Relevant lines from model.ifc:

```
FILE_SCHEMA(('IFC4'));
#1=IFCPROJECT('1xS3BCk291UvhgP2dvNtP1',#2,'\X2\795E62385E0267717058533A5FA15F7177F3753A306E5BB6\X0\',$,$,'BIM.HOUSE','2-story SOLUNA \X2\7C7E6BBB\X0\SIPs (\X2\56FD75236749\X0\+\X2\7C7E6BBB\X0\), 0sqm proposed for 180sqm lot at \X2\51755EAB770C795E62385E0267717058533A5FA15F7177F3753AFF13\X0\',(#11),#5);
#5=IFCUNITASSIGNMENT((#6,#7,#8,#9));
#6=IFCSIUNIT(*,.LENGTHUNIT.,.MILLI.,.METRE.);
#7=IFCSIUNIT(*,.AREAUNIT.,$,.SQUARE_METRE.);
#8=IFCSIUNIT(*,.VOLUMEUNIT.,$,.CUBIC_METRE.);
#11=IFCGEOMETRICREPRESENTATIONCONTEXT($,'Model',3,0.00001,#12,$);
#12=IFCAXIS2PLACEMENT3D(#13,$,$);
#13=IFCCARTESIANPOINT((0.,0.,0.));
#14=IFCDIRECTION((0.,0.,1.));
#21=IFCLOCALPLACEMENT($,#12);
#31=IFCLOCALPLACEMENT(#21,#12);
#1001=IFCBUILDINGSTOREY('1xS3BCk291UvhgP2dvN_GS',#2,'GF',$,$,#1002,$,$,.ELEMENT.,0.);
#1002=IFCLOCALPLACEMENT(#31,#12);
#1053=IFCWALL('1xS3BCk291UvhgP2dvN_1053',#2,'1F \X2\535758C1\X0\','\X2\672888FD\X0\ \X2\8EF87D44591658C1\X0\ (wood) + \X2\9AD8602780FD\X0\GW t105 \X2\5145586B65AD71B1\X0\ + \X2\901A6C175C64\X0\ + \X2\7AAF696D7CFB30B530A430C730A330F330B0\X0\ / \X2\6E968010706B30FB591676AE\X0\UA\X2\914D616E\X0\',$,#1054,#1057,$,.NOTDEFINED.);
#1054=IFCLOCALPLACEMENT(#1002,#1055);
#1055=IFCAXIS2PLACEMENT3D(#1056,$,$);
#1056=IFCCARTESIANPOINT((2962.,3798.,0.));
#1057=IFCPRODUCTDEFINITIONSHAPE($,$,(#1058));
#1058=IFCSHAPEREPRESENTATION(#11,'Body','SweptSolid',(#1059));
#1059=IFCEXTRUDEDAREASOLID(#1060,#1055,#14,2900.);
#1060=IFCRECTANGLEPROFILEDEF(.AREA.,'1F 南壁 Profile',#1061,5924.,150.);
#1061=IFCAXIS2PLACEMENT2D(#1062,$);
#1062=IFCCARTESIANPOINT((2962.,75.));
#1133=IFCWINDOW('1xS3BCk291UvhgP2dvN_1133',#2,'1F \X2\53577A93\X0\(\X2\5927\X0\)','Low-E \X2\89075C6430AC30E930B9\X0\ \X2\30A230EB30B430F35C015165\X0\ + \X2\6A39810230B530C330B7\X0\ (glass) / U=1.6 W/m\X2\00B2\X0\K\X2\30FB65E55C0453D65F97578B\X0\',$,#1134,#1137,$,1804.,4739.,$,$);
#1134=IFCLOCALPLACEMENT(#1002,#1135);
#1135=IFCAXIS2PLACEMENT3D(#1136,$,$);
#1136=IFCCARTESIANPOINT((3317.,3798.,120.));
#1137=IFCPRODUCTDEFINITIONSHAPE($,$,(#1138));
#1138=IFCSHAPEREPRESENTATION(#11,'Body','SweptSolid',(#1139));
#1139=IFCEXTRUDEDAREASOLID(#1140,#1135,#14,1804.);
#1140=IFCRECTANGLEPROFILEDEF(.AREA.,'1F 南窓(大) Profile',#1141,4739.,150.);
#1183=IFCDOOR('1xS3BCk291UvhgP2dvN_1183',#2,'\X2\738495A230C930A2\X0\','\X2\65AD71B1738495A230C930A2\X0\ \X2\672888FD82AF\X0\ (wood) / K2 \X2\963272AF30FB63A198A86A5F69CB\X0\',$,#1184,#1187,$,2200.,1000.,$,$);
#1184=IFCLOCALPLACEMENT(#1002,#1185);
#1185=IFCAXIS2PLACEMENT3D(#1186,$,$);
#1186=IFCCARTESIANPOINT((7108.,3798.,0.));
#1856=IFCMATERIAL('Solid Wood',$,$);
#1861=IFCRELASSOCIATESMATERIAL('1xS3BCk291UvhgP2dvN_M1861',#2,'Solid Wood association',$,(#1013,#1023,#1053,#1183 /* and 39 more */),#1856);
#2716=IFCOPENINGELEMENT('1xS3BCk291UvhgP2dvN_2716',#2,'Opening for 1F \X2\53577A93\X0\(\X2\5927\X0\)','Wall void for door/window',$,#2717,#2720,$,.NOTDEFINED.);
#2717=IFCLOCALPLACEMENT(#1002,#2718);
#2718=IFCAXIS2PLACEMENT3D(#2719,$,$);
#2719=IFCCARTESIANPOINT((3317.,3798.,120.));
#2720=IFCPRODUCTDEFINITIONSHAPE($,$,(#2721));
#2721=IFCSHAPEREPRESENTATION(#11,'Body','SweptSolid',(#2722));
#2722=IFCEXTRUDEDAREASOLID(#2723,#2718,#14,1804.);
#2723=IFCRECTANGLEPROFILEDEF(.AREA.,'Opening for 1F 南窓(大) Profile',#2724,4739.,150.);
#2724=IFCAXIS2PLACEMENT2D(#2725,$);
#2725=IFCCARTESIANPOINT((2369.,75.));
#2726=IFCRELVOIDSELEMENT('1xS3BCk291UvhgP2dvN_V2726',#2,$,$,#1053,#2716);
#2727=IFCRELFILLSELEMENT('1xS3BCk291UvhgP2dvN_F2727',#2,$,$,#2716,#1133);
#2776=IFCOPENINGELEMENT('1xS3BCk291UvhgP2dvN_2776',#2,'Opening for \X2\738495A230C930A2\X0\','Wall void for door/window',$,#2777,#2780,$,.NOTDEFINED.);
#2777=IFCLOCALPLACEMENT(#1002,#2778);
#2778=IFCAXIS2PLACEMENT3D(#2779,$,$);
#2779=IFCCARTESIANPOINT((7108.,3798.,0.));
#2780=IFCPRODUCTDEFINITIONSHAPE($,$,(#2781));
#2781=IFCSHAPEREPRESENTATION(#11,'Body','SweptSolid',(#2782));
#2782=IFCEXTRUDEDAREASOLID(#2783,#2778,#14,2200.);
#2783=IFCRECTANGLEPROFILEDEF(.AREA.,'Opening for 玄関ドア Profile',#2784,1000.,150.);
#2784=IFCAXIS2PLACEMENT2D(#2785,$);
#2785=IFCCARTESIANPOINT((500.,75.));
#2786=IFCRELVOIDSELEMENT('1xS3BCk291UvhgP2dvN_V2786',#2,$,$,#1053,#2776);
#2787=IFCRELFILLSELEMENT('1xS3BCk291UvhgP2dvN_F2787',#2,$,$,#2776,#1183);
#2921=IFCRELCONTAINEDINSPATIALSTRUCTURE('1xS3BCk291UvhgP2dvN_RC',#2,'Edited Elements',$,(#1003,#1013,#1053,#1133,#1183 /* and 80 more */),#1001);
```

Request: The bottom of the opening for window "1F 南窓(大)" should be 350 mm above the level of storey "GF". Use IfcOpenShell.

```python
import numpy as np
import ifcopenshell
import ifcopenshell.api.geometry
import ifcopenshell.geom
import ifcopenshell.util.element
import ifcopenshell.util.placement
import ifcopenshell.util.shape
import ifcopenshell.util.unit

model = ifcopenshell.open("model.ifc")
unit_scale = ifcopenshell.util.unit.calculate_unit_scale(model)

window = model.by_id(1133)
opening = window.FillsVoids[0].RelatingOpeningElement
storey = ifcopenshell.util.element.get_container(window, ifc_class="IfcBuildingStorey")
level = ifcopenshell.util.placement.get_local_placement(storey.ObjectPlacement)[2, 3]

# The opening's origin need not be at the sill, so measure its lowest point.
shape = ifcopenshell.geom.create_shape(ifcopenshell.geom.settings(), opening)
bottom = ifcopenshell.util.shape.get_shape_bottom_elevation(shape, shape.geometry) / unit_scale
dz = level + 0.35 / unit_scale - bottom

shift = np.array([0.0, 0.0, dz])
# The window is not placed relative to its opening, so move both.
for product in (opening, window):
    matrix = ifcopenshell.util.placement.get_local_placement(product.ObjectPlacement)
    matrix[:3, 3] += shift
    ifcopenshell.api.geometry.edit_object_placement(model, product=product, matrix=matrix, is_si=False)

print(f"moved by {dz * unit_scale:+.3f} m")

model.write("model_v2.ifc")
```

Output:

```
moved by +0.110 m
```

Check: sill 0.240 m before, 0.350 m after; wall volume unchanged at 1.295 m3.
